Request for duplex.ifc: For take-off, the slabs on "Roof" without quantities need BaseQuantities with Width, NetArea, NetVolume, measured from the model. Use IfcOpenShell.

First a look at what the model holds.

```python
import ifcopenshell
import ifcopenshell.util.element
import ifcopenshell.util.unit

model = ifcopenshell.open("duplex.ifc")
print(model.schema)
for unit_type in ("LENGTHUNIT", "AREAUNIT", "VOLUMEUNIT"):
    print(unit_type, ifcopenshell.util.unit.calculate_unit_scale(model, unit_type))
storey = next(s for s in model.by_type("IfcBuildingStorey") if s.Name == "Roof")
slabs = [e for e in ifcopenshell.util.element.get_decomposition(storey) if e.is_a("IfcSlab")]
for e in sorted(slabs, key=lambda e: e.id()):
    print(e.id(), e.is_a(), e.Name, list(ifcopenshell.util.element.get_psets(e, qtos_only=True)), sep=" | ")
```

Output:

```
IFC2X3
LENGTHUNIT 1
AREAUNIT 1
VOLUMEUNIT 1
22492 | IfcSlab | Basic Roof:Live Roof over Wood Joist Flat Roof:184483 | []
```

```python
import ifcopenshell
import ifcopenshell.api.pset
import ifcopenshell.geom
import ifcopenshell.util.element
import ifcopenshell.util.shape
import ifcopenshell.util.unit

model = ifcopenshell.open("duplex.ifc")
unit_scale = ifcopenshell.util.unit.calculate_unit_scale(model)
area_scale = ifcopenshell.util.unit.calculate_unit_scale(model, "AREAUNIT")
volume_scale = ifcopenshell.util.unit.calculate_unit_scale(model, "VOLUMEUNIT")
settings = ifcopenshell.geom.settings()

storey = next(s for s in model.by_type("IfcBuildingStorey") if s.Name == "Roof")
slabs = [e for e in ifcopenshell.util.element.get_decomposition(storey) if e.is_a("IfcSlab")]

for e in sorted(slabs, key=lambda e: e.id()):
    if ifcopenshell.util.element.get_psets(e, qtos_only=True, should_inherit=False):
        continue
    # Geometry comes back in metres, in the element's own axes.
    shape = ifcopenshell.geom.create_shape(settings, e)
    values = {
        "Width": ifcopenshell.util.shape.get_z(shape.geometry) / unit_scale,
        "NetArea": ifcopenshell.util.shape.get_footprint_area(shape.geometry) / area_scale,
        "NetVolume": ifcopenshell.util.shape.get_volume(shape.geometry) / volume_scale,
    }
    qto = ifcopenshell.api.pset.add_qto(model, product=e, name="BaseQuantities")
    ifcopenshell.api.pset.edit_qto(model, qto=qto, properties=values)
    print(e.id(), {k: round(v, 3) for k, v in values.items()})

model.write("duplex-out.ifc")
```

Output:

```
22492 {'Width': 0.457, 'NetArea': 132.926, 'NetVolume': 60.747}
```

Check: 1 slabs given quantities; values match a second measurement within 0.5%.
